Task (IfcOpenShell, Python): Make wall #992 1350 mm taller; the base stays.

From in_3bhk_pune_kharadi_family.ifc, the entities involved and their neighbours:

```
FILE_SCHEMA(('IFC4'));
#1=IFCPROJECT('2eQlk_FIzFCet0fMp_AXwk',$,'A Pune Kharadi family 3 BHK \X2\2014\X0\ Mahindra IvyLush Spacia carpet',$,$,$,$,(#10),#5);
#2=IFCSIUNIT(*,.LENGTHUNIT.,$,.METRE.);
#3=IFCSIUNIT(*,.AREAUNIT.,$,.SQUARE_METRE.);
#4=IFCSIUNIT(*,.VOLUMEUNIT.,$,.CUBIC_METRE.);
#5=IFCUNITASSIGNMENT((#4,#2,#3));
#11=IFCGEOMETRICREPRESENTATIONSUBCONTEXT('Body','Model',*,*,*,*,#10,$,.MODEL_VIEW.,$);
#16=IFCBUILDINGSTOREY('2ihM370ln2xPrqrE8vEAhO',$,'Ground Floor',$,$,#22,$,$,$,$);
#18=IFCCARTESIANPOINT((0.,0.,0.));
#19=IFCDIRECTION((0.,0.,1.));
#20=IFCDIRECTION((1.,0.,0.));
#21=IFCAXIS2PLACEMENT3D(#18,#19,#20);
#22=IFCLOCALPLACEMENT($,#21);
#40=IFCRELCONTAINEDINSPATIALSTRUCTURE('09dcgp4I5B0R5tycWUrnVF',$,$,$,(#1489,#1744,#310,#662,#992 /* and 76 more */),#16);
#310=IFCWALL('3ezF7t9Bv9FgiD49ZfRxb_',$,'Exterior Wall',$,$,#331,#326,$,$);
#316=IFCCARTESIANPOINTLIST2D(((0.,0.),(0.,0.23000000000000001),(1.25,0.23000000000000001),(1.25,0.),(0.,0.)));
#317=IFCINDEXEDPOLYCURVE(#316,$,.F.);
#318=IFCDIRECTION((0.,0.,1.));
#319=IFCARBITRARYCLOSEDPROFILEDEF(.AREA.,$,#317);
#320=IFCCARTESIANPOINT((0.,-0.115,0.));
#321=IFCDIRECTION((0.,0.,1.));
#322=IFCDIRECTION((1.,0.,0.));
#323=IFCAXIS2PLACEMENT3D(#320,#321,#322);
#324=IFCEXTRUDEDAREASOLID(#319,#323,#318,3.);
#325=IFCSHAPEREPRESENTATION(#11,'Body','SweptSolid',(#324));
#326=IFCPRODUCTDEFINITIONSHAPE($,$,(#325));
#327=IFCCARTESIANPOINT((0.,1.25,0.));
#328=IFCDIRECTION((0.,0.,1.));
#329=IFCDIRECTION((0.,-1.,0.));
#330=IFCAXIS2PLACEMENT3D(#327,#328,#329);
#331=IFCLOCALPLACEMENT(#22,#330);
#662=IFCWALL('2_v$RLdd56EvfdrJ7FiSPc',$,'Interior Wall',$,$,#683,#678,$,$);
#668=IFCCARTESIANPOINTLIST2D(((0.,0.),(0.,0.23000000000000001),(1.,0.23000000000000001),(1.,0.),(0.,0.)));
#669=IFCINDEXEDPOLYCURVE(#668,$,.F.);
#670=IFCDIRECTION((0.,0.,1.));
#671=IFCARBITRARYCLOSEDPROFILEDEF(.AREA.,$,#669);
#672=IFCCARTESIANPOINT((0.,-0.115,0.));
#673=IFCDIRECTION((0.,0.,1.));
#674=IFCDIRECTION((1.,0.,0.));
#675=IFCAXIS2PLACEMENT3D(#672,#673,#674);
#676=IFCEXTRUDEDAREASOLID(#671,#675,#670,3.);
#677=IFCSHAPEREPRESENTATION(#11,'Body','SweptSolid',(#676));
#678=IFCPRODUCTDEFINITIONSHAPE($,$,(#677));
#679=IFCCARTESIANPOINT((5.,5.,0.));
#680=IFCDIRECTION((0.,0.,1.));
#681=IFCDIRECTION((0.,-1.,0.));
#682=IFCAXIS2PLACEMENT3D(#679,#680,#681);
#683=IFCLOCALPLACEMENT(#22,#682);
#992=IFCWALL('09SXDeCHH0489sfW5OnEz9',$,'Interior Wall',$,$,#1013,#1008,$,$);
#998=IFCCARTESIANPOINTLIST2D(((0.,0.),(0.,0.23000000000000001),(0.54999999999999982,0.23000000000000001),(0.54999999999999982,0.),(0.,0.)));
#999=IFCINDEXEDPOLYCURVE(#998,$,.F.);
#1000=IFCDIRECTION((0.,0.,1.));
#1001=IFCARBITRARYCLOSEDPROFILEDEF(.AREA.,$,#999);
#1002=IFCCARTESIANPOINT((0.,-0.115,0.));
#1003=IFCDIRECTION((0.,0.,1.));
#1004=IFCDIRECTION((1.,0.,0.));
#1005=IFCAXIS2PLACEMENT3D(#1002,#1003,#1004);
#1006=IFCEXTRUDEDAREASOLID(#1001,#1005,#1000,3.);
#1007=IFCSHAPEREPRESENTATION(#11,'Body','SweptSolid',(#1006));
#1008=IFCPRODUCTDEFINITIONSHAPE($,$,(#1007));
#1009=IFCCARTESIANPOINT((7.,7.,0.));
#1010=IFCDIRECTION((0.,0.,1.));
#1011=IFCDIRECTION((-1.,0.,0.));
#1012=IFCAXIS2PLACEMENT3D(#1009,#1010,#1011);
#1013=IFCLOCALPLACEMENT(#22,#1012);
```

```python
import ifcopenshell
import ifcopenshell.geom
import ifcopenshell.util.representation
import ifcopenshell.util.shape

model = ifcopenshell.open("in_3bhk_pune_kharadi_family.ifc")
settings = ifcopenshell.geom.settings()


def volume(element):
    """Net volume in cubic metres, openings subtracted."""
    shape = ifcopenshell.geom.create_shape(settings, element)
    return ifcopenshell.util.shape.get_volume(shape.geometry)


wall = model.by_guid("09SXDeCHH0489sfW5OnEz9")
before = volume(wall)

body = ifcopenshell.util.representation.get_representation(wall, "Model", "Body")
solid = body.Items[0]
old_height = solid.Depth
solid.Depth += 1.35
after = volume(wall)

print(f"height {old_height:g} -> {solid.Depth:g}, volume {before:.3f} -> {after:.3f} m3")

model.write("in_3bhk_pune_kharadi_family_v2.ifc")
```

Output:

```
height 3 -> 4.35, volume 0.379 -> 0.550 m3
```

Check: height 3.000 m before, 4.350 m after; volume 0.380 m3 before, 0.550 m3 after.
